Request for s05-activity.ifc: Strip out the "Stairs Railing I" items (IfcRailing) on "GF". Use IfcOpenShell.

First a look at what the model holds.

```python
import ifcopenshell
import ifcopenshell.util.element

model = ifcopenshell.open("s05-activity.ifc")
print(model.schema)
storey = next(s for s in model.by_type("IfcBuildingStorey") if s.Name == "GF")
railings = [e for e in ifcopenshell.util.element.get_decomposition(storey) if e.is_a("IfcRailing")]
seen = {}
for e in railings:
    element_type = ifcopenshell.util.element.get_type(e)
    name = element_type.Name if element_type not in (None, e) else None
    seen[name] = seen.get(name, 0) + 1
for name, count in sorted(seen.items(), key=str):
    print(count, "x", name)
```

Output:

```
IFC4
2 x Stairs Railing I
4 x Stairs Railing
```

```python
import ifcopenshell
import ifcopenshell.api.root
import ifcopenshell.util.element

model = ifcopenshell.open("s05-activity.ifc")

storey = next(s for s in model.by_type("IfcBuildingStorey") if s.Name == "GF")
railings = [e for e in ifcopenshell.util.element.get_decomposition(storey) if e.is_a("IfcRailing")]
targets = [e for e in railings if (t := ifcopenshell.util.element.get_type(e)) not in (None, e) and t.Name == "Stairs Railing I"]

for e in targets:
    ifcopenshell.api.root.remove_product(model, product=e)
print(len(targets), "removed")

model.write("s05-activity-out.ifc")
```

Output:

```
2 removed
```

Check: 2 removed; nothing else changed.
